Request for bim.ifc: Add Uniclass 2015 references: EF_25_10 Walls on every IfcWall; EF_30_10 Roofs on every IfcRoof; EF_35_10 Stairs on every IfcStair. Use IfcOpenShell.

First a look at what the model holds.

```python
import ifcopenshell

model = ifcopenshell.open("bim.ifc")
print(model.schema)
print("classifications:", [c.Name for c in model.by_type("IfcClassification")])
for ifc_class in ("IfcDoor", "IfcRoof", "IfcStair", "IfcWall", "IfcWindow"):
    print(ifc_class, len(model.by_type(ifc_class)))
```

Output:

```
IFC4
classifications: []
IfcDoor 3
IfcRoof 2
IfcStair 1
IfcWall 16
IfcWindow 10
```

```python
import ifcopenshell
import ifcopenshell.api.classification

model = ifcopenshell.open("bim.ifc")

system = ifcopenshell.api.classification.add_classification(model, classification="Uniclass 2015")

codes = {
    "IfcWall": ("EF_25_10", "Walls"),
    "IfcRoof": ("EF_30_10", "Roofs"),
    "IfcStair": ("EF_35_10", "Stairs"),
}
for ifc_class, (code, name) in codes.items():
    products = model.by_type(ifc_class)
    ifcopenshell.api.classification.add_reference(
        model, products=products, classification=system, identification=code, name=name
    )
    print(code, len(products))

model.write("bim_updated.ifc")
```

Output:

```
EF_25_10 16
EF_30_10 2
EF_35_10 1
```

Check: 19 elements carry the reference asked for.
